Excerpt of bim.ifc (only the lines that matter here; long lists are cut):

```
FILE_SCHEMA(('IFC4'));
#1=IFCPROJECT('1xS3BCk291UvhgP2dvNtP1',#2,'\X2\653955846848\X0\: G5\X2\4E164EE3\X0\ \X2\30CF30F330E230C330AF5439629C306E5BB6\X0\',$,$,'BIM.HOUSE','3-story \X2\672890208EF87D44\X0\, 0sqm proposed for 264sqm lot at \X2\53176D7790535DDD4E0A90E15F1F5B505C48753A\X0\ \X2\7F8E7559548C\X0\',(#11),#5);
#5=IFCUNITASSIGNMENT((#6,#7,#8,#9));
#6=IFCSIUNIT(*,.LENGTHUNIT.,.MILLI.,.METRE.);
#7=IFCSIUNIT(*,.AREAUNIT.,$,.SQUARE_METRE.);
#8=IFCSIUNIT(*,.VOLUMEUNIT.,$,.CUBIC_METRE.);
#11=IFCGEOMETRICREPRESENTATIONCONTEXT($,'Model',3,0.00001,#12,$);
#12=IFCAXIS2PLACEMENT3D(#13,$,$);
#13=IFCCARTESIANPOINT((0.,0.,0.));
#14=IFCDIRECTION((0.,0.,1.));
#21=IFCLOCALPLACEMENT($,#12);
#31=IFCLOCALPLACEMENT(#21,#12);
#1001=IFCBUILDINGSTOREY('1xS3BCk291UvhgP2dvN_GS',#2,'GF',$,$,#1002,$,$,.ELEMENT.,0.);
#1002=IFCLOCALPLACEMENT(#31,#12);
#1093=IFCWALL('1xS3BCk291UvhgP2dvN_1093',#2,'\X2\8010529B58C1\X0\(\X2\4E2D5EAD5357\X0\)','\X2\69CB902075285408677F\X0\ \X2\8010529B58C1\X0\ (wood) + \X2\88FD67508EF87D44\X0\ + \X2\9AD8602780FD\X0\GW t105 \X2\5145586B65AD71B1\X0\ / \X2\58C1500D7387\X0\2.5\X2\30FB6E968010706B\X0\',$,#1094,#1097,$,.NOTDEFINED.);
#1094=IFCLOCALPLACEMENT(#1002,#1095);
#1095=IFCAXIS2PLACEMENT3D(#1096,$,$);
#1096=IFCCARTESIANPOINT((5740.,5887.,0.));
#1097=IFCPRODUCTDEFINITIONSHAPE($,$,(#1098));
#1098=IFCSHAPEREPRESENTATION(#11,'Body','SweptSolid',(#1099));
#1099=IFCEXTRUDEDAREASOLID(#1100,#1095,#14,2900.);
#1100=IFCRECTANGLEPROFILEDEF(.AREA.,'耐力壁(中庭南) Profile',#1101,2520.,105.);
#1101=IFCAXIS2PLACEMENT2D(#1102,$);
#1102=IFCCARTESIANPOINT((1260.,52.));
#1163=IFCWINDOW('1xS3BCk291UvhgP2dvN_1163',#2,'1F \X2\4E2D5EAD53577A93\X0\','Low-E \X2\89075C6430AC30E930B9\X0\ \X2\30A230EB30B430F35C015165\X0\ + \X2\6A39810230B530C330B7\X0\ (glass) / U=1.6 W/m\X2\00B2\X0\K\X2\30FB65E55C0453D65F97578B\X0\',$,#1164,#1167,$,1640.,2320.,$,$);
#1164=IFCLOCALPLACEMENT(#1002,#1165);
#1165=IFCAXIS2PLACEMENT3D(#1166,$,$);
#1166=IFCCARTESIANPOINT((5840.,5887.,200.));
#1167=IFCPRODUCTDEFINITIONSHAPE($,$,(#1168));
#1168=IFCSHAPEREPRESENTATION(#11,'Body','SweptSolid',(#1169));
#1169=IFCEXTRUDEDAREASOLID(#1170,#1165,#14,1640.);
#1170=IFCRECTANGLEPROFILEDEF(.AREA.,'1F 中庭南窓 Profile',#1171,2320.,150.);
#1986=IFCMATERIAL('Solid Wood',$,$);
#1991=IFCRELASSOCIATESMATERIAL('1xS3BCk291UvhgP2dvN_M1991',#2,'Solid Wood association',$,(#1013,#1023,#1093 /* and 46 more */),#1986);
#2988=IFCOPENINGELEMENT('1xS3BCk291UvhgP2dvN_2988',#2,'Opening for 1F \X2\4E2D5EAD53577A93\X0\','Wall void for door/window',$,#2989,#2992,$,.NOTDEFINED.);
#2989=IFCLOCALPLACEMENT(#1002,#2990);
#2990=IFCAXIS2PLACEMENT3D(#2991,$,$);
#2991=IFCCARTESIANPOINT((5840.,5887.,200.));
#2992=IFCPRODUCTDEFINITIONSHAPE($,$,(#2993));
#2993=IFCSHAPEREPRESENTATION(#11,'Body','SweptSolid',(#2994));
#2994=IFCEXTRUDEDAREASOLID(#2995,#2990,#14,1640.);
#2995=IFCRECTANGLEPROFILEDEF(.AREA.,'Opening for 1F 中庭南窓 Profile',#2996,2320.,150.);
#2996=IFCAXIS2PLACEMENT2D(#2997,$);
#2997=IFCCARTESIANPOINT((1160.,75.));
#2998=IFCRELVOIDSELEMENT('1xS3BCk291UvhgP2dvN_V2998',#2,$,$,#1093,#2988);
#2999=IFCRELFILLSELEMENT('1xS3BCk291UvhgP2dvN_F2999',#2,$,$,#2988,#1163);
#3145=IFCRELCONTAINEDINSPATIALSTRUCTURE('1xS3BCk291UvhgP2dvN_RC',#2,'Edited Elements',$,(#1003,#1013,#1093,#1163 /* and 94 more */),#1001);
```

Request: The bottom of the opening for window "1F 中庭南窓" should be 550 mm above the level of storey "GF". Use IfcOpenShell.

```python
import numpy as np
import ifcopenshell
import ifcopenshell.api.geometry
import ifcopenshell.geom
import ifcopenshell.util.element
import ifcopenshell.util.placement
import ifcopenshell.util.shape
import ifcopenshell.util.unit

model = ifcopenshell.open("bim.ifc")
unit_scale = ifcopenshell.util.unit.calculate_unit_scale(model)

window = model.by_id(1163)
opening = window.FillsVoids[0].RelatingOpeningElement
storey = ifcopenshell.util.element.get_container(window, ifc_class="IfcBuildingStorey")
level = ifcopenshell.util.placement.get_local_placement(storey.ObjectPlacement)[2, 3]

# The opening's origin need not be at the sill, so measure its lowest point.
shape = ifcopenshell.geom.create_shape(ifcopenshell.geom.settings(), opening)
bottom = ifcopenshell.util.shape.get_shape_bottom_elevation(shape, shape.geometry) / unit_scale
dz = level + 0.55 / unit_scale - bottom

shift = np.array([0.0, 0.0, dz])
# The window is not placed relative to its opening, so move both.
for product in (opening, window):
    matrix = ifcopenshell.util.placement.get_local_placement(product.ObjectPlacement)
    matrix[:3, 3] += shift
    ifcopenshell.api.geometry.edit_object_placement(model, product=product, matrix=matrix, is_si=False)

print(f"moved by {dz * unit_scale:+.3f} m")

model.write("bim_rev.ifc")
```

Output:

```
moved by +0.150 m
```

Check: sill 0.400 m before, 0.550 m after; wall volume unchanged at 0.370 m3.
